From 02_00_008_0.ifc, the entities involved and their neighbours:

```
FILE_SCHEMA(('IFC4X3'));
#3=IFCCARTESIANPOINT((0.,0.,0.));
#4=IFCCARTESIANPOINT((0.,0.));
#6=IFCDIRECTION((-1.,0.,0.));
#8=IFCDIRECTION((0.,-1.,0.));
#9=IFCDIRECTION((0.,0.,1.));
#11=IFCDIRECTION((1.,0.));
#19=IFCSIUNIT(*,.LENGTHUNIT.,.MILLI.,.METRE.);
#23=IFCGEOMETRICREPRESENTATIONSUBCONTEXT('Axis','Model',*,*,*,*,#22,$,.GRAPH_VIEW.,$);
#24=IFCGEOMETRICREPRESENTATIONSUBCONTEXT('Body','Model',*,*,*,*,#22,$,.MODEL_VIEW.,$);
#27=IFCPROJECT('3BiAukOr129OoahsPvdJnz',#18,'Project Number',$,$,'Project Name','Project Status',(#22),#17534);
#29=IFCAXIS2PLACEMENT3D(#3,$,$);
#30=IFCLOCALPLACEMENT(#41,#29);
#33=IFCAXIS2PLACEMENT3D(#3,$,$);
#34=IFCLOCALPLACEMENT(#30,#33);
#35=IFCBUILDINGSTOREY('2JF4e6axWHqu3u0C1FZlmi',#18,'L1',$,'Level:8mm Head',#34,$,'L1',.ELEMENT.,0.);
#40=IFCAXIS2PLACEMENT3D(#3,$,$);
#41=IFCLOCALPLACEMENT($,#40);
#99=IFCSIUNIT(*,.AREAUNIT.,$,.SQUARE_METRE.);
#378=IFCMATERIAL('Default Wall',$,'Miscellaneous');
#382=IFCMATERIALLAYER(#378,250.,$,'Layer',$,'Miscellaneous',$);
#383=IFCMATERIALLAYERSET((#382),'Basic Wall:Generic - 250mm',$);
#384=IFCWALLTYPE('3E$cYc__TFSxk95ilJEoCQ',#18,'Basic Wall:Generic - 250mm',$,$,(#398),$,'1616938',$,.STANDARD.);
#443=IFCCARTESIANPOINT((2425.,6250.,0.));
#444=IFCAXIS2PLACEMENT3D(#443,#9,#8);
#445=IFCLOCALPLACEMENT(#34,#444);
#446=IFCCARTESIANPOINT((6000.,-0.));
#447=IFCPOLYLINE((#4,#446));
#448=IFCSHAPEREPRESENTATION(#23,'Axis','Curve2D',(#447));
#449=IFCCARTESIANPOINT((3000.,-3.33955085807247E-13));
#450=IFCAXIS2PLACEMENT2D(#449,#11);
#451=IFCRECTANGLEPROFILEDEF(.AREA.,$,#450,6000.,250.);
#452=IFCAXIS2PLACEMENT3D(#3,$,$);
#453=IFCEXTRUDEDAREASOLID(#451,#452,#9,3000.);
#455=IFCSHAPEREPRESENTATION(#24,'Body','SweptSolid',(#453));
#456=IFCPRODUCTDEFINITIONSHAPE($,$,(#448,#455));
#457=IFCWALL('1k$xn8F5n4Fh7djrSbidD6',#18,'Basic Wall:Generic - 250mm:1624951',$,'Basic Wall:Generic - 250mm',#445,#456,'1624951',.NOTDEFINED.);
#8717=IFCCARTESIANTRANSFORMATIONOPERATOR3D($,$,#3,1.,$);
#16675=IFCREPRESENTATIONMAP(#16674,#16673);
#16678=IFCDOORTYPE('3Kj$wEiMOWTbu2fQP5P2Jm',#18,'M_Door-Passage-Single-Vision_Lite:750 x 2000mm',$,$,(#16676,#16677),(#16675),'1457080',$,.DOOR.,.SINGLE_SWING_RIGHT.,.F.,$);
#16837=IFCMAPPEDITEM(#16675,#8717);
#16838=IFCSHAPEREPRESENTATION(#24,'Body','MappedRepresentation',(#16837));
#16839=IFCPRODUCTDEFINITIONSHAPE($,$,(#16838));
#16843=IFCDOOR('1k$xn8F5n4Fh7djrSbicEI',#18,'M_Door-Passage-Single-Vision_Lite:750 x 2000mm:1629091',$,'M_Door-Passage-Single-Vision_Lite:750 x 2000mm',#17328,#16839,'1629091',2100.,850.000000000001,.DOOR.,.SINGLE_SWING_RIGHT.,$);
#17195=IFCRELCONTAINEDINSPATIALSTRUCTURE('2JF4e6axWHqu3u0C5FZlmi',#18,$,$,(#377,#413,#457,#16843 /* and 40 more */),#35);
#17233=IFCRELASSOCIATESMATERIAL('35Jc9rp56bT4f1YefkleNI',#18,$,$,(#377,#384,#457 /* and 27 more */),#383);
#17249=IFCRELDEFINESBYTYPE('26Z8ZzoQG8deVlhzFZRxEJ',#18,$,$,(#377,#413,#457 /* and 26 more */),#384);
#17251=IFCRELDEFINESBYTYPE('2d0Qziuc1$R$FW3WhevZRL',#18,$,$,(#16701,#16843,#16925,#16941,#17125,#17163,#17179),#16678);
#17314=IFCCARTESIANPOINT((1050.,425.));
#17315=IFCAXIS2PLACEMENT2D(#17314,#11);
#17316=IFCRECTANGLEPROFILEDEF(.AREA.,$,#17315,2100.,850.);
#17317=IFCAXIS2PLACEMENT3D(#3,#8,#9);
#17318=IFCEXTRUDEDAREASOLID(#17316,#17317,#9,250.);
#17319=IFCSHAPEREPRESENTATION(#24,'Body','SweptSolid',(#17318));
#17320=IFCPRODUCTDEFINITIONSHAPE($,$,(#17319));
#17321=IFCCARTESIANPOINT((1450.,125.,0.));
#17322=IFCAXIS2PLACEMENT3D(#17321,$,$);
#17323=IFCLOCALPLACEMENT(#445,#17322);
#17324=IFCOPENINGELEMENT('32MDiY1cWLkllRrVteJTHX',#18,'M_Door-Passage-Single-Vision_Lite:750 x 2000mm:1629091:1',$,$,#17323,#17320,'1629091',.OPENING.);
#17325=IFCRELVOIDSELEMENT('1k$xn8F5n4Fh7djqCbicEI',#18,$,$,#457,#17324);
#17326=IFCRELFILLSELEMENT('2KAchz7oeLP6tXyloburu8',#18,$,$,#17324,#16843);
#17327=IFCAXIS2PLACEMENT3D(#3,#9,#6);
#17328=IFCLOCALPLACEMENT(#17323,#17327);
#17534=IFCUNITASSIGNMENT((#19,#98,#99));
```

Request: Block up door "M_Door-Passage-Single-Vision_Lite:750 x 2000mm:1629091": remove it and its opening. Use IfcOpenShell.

```python
import ifcopenshell
import ifcopenshell.api.feature
import ifcopenshell.api.root
import ifcopenshell.geom
import ifcopenshell.util.shape

model = ifcopenshell.open("02_00_008_0.ifc")
settings = ifcopenshell.geom.settings()


def volume(element):
    """Net volume in cubic metres, openings subtracted."""
    shape = ifcopenshell.geom.create_shape(settings, element)
    return ifcopenshell.util.shape.get_volume(shape.geometry)


door = model.by_guid("1k$xn8F5n4Fh7djrSbicEI")
opening = door.FillsVoids[0].RelatingOpeningElement
wall = opening.VoidsElements[0].RelatingBuildingElement
before = volume(wall)

ifcopenshell.api.root.remove_product(model, product=door)
ifcopenshell.api.feature.remove_feature(model, feature=opening)

after = volume(wall)

print(f"wall volume {before:.3f} -> {after:.3f} m3")

model.write("02_00_008_0-out.ifc")
```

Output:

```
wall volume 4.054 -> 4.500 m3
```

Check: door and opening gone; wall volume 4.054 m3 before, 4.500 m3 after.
